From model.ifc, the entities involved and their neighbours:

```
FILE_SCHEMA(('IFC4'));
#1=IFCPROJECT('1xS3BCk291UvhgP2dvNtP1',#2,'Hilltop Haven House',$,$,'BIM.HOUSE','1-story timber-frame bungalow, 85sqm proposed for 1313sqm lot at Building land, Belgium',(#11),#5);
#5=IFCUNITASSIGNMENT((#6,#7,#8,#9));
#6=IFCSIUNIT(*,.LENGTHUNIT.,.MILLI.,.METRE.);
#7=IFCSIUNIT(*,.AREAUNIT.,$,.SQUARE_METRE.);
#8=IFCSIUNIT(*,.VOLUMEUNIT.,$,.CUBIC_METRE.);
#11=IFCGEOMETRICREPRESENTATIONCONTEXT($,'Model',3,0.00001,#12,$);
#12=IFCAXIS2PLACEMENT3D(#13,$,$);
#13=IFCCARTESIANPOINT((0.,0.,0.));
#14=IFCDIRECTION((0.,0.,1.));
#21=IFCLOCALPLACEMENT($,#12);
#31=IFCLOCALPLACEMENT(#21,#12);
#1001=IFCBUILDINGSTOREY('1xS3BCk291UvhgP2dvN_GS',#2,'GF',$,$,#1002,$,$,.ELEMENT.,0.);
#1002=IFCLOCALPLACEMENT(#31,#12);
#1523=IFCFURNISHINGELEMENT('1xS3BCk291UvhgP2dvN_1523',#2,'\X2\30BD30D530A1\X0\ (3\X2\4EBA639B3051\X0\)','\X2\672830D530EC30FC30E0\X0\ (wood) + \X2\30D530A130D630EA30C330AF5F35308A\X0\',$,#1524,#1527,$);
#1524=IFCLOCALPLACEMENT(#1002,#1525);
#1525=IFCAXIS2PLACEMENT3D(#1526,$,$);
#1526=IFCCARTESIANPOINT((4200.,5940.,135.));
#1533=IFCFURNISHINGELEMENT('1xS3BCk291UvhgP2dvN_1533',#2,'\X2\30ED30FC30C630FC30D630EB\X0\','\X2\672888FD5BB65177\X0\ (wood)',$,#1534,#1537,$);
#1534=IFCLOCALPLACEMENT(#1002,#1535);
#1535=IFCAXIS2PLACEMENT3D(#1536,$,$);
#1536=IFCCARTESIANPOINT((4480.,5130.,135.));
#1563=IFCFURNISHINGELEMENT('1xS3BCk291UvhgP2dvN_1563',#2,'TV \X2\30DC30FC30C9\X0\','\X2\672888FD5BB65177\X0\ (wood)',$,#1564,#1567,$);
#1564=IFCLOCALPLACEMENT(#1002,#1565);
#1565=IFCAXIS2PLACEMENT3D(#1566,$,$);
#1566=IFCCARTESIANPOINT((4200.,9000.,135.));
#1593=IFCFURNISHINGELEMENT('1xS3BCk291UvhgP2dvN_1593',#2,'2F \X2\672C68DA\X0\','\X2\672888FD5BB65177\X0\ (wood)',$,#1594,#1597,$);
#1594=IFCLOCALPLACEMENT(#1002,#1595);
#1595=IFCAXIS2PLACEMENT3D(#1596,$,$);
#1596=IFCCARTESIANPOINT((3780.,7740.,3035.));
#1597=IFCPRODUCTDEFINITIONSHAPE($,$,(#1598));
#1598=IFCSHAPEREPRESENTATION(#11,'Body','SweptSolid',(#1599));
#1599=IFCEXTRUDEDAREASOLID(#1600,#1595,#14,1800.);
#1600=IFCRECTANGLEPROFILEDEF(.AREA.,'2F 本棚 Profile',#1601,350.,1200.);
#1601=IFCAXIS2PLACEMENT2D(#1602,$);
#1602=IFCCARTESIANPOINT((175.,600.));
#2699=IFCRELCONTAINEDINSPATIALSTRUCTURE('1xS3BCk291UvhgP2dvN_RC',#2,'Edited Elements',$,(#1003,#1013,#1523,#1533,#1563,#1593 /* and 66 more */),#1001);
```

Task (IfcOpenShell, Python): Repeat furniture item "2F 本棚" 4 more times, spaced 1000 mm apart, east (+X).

```python
import numpy as np
import ifcopenshell
import ifcopenshell.api.geometry
import ifcopenshell.api.root
import ifcopenshell.util.element
import ifcopenshell.util.placement

model = ifcopenshell.open("model.ifc")


def reuse_history(source, copy):
    """copy_class also copies each property set's owner history, people and application; keep the originals."""
    for rel in copy.IsDefinedBy:
        if rel.is_a("IfcRelDefinesByProperties") and (history := rel.RelatingPropertyDefinition.OwnerHistory):
            rel.RelatingPropertyDefinition.OwnerHistory = source.OwnerHistory
            ifcopenshell.util.element.remove_deep2(model, history)


source = model.by_guid("1xS3BCk291UvhgP2dvN_1593")
base = ifcopenshell.util.placement.get_local_placement(source.ObjectPlacement)
step = np.array([1.0, 0.0, 0.0]) * 1000.0

for i in range(1, 5):
    copy = ifcopenshell.api.root.copy_class(model, product=source)
    copy.Representation = ifcopenshell.util.element.copy_deep(
        model, source.Representation, exclude=["IfcGeometricRepresentationContext", "IfcRepresentationMap"]
    )
    reuse_history(source, copy)
    matrix = base.copy()
    matrix[:3, 3] += i * step
    print("added at", matrix[:3, 3].round(3) + 0.0)
    ifcopenshell.api.geometry.edit_object_placement(model, product=copy, matrix=matrix, is_si=False)

model.write("model_v2.ifc")
```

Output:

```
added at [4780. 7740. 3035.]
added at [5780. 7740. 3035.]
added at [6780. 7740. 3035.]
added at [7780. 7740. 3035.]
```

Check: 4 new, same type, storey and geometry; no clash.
